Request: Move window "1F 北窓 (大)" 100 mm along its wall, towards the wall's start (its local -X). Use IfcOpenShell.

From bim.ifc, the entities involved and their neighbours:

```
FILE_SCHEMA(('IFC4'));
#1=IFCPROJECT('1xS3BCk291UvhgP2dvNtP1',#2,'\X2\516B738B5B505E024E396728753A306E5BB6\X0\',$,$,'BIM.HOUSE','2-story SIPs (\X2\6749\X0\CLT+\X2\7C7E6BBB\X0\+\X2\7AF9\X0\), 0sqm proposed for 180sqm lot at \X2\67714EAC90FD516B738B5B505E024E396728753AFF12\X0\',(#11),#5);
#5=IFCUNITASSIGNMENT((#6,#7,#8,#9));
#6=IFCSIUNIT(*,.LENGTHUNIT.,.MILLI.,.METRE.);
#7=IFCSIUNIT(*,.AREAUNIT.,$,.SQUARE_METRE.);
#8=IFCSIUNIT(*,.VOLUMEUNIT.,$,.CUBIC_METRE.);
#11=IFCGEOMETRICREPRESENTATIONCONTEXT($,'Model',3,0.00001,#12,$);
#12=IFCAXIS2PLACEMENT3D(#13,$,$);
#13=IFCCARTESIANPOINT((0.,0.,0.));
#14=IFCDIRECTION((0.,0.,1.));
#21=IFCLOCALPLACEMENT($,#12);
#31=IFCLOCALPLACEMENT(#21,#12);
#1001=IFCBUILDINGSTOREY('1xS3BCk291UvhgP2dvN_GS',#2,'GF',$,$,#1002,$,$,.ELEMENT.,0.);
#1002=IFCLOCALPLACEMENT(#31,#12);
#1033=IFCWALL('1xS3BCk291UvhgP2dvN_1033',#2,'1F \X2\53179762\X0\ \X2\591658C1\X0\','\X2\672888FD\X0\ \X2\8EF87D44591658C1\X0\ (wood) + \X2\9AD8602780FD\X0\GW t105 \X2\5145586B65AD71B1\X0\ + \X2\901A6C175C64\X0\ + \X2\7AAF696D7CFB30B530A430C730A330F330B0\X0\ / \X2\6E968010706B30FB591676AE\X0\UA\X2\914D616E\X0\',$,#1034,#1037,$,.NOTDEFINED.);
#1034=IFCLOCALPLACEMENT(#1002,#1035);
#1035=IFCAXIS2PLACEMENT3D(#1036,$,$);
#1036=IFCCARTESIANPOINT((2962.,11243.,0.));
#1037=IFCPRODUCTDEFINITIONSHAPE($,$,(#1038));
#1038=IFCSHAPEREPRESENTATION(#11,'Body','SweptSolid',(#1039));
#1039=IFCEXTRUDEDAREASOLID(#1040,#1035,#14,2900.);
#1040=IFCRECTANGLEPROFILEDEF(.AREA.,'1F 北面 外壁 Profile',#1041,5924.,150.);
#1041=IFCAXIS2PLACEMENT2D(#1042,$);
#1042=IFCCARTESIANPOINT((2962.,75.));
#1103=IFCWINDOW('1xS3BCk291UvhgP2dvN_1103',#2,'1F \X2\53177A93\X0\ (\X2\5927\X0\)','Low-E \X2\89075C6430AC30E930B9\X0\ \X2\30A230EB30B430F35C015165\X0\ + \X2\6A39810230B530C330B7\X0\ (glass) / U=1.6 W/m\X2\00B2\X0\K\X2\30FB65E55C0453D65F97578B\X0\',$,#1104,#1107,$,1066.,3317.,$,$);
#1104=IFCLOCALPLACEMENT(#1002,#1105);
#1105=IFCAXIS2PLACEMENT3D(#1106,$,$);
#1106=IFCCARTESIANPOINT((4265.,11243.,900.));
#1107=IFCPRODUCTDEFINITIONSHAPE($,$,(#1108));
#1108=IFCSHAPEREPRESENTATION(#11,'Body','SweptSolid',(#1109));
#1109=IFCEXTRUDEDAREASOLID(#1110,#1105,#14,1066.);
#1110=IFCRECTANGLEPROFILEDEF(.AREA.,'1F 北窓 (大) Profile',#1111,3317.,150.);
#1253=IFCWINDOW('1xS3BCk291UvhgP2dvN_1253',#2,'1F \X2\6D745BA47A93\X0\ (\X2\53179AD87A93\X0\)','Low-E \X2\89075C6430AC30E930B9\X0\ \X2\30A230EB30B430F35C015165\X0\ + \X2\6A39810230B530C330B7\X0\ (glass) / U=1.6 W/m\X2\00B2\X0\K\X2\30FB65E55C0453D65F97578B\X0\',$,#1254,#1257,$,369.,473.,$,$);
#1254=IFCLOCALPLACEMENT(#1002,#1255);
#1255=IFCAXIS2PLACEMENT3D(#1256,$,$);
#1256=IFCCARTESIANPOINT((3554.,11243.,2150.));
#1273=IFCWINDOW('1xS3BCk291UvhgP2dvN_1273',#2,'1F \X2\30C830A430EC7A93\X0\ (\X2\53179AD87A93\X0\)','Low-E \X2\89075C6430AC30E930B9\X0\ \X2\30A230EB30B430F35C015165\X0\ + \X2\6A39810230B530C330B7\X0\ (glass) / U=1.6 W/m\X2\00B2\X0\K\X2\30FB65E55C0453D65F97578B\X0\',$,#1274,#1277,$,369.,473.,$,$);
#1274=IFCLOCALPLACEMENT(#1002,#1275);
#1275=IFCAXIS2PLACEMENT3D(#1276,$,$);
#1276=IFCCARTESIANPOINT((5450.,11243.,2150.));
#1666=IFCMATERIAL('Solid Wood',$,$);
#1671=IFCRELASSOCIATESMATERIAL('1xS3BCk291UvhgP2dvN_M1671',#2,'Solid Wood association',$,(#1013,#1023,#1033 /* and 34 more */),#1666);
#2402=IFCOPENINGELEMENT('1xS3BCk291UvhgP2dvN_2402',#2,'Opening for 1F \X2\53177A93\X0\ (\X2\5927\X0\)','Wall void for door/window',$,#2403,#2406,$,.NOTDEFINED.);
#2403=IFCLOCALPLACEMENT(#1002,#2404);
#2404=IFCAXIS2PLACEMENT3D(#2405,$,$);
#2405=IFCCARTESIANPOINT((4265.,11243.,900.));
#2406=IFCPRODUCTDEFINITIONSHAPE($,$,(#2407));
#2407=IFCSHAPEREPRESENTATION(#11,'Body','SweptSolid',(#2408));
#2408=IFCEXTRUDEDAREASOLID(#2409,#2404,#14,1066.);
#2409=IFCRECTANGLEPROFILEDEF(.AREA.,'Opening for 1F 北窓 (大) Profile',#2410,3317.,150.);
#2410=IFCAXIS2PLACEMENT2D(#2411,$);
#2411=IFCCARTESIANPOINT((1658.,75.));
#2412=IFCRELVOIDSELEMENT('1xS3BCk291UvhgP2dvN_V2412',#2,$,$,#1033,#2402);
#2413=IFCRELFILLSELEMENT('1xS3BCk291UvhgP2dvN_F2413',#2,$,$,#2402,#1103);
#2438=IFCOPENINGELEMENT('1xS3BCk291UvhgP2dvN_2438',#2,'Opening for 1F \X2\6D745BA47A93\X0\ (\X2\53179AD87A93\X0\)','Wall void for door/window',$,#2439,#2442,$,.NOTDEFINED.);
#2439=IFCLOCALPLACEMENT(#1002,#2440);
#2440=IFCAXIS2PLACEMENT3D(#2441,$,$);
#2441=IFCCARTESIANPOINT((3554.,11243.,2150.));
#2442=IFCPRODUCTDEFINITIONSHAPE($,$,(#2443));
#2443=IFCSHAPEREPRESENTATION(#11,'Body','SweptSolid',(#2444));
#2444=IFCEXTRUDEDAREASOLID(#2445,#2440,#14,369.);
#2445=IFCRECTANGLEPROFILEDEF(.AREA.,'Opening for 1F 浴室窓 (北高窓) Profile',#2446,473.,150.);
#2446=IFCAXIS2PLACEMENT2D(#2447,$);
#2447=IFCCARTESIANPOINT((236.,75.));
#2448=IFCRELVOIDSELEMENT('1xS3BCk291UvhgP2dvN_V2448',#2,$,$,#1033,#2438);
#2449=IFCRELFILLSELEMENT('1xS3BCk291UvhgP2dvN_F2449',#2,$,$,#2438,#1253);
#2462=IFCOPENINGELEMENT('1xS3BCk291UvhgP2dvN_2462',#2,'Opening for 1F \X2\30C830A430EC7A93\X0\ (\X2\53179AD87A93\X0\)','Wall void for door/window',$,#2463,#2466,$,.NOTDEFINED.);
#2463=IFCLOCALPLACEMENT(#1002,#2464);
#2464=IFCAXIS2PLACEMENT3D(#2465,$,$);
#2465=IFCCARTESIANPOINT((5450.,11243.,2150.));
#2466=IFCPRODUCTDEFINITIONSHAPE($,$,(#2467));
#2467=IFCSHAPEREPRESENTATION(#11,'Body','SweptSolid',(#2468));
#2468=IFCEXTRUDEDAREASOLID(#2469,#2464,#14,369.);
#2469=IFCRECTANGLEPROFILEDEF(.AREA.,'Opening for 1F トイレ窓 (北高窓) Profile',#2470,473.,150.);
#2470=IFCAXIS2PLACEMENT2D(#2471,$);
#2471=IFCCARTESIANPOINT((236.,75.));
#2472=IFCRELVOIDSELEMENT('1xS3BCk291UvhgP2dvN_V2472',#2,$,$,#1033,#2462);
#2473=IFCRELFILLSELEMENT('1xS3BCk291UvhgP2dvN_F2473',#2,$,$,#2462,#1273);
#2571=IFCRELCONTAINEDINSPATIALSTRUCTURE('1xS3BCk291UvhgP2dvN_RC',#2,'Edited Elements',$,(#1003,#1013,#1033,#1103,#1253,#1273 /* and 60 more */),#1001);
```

```python
import ifcopenshell
import ifcopenshell.api.geometry
import ifcopenshell.util.placement

model = ifcopenshell.open("bim.ifc")

window = model.by_guid("1xS3BCk291UvhgP2dvN_1103")
opening = window.FillsVoids[0].RelatingOpeningElement
wall = opening.VoidsElements[0].RelatingBuildingElement

wall_matrix = ifcopenshell.util.placement.get_local_placement(wall.ObjectPlacement)
shift = wall_matrix[:3, 0] * -100.0
before = ifcopenshell.util.placement.get_local_placement(window.ObjectPlacement)[:3, 3].copy()

# The window is not placed relative to its opening, so move both.
for product in (opening, window):
    matrix = ifcopenshell.util.placement.get_local_placement(product.ObjectPlacement)
    matrix[:3, 3] += shift
    ifcopenshell.api.geometry.edit_object_placement(model, product=product, matrix=matrix, is_si=False)

after = ifcopenshell.util.placement.get_local_placement(window.ObjectPlacement)[:3, 3]
print("window moved by", (after - before).round(3) + 0.0)

model.write("bim-out.ifc")
```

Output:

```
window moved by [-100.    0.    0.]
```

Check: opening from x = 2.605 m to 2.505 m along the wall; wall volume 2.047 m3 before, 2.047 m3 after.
